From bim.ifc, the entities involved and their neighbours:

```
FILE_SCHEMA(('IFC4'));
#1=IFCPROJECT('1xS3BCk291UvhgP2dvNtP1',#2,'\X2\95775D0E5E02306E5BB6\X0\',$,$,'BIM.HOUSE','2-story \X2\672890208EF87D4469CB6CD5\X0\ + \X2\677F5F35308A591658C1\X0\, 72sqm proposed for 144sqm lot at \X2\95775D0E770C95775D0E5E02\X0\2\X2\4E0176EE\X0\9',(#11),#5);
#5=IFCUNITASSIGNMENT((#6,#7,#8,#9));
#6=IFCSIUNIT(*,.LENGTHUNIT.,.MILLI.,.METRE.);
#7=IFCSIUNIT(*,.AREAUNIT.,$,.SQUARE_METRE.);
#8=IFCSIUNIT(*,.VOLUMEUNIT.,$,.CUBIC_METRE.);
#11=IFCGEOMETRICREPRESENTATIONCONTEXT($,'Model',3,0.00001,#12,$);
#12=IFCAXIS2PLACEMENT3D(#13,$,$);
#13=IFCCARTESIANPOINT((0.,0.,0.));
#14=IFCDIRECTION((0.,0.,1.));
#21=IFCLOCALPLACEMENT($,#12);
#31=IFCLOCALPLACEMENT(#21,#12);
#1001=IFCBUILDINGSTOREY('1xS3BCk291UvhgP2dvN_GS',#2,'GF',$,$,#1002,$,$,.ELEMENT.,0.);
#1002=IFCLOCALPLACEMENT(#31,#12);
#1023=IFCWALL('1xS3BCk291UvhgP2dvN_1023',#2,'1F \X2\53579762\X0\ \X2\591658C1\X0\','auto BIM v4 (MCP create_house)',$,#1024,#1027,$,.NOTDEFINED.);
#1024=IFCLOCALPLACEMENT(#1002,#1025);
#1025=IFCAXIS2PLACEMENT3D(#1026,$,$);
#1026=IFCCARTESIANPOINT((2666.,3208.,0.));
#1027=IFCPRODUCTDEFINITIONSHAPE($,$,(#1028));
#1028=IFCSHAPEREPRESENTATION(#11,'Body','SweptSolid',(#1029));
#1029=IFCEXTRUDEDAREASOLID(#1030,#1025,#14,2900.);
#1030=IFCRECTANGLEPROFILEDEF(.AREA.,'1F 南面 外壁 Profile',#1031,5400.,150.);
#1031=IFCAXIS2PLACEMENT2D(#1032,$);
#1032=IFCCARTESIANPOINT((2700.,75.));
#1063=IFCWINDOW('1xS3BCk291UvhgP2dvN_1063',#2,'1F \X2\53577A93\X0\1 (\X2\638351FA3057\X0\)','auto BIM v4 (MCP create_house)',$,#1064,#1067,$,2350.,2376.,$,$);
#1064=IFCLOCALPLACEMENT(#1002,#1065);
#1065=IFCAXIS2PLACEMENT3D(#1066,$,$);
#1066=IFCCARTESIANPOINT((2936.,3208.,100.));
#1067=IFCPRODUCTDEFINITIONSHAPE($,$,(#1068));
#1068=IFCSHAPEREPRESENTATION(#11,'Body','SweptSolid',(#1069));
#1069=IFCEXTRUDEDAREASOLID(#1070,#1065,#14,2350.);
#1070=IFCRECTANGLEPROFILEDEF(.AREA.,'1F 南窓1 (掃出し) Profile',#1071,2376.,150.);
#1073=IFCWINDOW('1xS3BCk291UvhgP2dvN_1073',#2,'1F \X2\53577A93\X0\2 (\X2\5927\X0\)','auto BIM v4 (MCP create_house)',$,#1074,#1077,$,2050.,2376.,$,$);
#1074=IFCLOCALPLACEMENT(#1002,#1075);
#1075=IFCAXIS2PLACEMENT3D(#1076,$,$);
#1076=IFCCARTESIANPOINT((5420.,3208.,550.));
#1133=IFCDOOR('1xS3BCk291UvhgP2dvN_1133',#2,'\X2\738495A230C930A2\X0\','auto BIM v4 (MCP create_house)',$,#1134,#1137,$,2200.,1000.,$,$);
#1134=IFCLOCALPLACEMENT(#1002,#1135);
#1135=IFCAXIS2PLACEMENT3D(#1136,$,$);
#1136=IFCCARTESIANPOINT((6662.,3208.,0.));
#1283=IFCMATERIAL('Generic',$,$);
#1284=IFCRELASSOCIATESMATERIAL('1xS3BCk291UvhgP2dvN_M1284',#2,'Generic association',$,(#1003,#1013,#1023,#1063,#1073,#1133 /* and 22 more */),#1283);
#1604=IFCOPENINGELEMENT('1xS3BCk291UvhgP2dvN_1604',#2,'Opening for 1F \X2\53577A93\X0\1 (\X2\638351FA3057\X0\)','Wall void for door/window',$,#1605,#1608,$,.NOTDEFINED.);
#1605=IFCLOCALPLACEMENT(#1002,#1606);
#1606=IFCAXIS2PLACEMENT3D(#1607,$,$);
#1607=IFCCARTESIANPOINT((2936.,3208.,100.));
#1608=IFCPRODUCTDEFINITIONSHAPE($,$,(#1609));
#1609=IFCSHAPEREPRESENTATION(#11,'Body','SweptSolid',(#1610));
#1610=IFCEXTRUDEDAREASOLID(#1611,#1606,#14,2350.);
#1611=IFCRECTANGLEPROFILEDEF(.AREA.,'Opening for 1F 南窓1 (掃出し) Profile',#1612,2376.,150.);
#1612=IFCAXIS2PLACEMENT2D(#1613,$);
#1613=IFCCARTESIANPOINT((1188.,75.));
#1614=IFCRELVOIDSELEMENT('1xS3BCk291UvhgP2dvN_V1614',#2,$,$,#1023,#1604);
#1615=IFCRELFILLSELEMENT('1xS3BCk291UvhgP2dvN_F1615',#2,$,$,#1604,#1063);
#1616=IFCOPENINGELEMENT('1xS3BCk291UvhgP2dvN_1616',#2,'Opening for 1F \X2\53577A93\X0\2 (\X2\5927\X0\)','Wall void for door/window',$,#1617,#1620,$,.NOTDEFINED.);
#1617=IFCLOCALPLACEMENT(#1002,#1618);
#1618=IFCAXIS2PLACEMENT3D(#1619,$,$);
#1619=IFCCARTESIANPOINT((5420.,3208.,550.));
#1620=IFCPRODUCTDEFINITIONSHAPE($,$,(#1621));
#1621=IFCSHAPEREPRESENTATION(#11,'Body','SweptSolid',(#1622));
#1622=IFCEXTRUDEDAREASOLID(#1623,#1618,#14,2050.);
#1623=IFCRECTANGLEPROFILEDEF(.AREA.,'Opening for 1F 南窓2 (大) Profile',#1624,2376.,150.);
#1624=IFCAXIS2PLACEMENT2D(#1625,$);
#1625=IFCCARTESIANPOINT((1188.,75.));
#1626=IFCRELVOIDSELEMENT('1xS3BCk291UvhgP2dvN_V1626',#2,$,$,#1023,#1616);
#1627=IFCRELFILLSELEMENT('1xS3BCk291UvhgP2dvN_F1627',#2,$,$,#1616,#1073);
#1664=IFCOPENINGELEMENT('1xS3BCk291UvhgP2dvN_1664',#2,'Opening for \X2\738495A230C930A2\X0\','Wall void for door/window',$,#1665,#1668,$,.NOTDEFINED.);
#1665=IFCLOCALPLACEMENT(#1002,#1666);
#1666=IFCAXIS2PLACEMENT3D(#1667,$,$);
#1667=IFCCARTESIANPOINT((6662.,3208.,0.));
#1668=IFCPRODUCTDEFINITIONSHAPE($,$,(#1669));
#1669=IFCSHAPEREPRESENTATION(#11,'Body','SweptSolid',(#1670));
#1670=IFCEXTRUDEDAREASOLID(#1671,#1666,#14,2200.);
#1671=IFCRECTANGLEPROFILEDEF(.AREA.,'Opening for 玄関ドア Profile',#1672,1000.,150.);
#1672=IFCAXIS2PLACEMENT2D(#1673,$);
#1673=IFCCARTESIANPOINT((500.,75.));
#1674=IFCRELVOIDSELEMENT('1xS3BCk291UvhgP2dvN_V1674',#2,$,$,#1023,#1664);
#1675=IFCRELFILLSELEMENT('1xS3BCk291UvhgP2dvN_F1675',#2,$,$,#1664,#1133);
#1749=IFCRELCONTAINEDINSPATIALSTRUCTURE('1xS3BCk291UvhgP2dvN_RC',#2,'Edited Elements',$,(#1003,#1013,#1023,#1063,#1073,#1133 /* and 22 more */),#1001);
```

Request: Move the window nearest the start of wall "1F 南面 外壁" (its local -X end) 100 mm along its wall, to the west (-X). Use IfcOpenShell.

```python
import ifcopenshell
import ifcopenshell.api.geometry
import ifcopenshell.util.placement
import ifcopenshell.util.unit

model = ifcopenshell.open("bim.ifc")
unit_scale = ifcopenshell.util.unit.calculate_unit_scale(model)

window = model.by_guid("1xS3BCk291UvhgP2dvN_1063")
opening = window.FillsVoids[0].RelatingOpeningElement
wall = opening.VoidsElements[0].RelatingBuildingElement

wall_matrix = ifcopenshell.util.placement.get_local_placement(wall.ObjectPlacement)
shift = wall_matrix[:3, 0] * -0.1 / unit_scale
before = ifcopenshell.util.placement.get_local_placement(window.ObjectPlacement)[:3, 3].copy()

# The window is not placed relative to its opening, so move both.
for product in (opening, window):
    matrix = ifcopenshell.util.placement.get_local_placement(product.ObjectPlacement)
    matrix[:3, 3] += shift
    ifcopenshell.api.geometry.edit_object_placement(model, product=product, matrix=matrix, is_si=False)

after = ifcopenshell.util.placement.get_local_placement(window.ObjectPlacement)[:3, 3]
print("window moved by", (after - before).round(3) + 0.0)

model.write("bim_v2.ifc")
```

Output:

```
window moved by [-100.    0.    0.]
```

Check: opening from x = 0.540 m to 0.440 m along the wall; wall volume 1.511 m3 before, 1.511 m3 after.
